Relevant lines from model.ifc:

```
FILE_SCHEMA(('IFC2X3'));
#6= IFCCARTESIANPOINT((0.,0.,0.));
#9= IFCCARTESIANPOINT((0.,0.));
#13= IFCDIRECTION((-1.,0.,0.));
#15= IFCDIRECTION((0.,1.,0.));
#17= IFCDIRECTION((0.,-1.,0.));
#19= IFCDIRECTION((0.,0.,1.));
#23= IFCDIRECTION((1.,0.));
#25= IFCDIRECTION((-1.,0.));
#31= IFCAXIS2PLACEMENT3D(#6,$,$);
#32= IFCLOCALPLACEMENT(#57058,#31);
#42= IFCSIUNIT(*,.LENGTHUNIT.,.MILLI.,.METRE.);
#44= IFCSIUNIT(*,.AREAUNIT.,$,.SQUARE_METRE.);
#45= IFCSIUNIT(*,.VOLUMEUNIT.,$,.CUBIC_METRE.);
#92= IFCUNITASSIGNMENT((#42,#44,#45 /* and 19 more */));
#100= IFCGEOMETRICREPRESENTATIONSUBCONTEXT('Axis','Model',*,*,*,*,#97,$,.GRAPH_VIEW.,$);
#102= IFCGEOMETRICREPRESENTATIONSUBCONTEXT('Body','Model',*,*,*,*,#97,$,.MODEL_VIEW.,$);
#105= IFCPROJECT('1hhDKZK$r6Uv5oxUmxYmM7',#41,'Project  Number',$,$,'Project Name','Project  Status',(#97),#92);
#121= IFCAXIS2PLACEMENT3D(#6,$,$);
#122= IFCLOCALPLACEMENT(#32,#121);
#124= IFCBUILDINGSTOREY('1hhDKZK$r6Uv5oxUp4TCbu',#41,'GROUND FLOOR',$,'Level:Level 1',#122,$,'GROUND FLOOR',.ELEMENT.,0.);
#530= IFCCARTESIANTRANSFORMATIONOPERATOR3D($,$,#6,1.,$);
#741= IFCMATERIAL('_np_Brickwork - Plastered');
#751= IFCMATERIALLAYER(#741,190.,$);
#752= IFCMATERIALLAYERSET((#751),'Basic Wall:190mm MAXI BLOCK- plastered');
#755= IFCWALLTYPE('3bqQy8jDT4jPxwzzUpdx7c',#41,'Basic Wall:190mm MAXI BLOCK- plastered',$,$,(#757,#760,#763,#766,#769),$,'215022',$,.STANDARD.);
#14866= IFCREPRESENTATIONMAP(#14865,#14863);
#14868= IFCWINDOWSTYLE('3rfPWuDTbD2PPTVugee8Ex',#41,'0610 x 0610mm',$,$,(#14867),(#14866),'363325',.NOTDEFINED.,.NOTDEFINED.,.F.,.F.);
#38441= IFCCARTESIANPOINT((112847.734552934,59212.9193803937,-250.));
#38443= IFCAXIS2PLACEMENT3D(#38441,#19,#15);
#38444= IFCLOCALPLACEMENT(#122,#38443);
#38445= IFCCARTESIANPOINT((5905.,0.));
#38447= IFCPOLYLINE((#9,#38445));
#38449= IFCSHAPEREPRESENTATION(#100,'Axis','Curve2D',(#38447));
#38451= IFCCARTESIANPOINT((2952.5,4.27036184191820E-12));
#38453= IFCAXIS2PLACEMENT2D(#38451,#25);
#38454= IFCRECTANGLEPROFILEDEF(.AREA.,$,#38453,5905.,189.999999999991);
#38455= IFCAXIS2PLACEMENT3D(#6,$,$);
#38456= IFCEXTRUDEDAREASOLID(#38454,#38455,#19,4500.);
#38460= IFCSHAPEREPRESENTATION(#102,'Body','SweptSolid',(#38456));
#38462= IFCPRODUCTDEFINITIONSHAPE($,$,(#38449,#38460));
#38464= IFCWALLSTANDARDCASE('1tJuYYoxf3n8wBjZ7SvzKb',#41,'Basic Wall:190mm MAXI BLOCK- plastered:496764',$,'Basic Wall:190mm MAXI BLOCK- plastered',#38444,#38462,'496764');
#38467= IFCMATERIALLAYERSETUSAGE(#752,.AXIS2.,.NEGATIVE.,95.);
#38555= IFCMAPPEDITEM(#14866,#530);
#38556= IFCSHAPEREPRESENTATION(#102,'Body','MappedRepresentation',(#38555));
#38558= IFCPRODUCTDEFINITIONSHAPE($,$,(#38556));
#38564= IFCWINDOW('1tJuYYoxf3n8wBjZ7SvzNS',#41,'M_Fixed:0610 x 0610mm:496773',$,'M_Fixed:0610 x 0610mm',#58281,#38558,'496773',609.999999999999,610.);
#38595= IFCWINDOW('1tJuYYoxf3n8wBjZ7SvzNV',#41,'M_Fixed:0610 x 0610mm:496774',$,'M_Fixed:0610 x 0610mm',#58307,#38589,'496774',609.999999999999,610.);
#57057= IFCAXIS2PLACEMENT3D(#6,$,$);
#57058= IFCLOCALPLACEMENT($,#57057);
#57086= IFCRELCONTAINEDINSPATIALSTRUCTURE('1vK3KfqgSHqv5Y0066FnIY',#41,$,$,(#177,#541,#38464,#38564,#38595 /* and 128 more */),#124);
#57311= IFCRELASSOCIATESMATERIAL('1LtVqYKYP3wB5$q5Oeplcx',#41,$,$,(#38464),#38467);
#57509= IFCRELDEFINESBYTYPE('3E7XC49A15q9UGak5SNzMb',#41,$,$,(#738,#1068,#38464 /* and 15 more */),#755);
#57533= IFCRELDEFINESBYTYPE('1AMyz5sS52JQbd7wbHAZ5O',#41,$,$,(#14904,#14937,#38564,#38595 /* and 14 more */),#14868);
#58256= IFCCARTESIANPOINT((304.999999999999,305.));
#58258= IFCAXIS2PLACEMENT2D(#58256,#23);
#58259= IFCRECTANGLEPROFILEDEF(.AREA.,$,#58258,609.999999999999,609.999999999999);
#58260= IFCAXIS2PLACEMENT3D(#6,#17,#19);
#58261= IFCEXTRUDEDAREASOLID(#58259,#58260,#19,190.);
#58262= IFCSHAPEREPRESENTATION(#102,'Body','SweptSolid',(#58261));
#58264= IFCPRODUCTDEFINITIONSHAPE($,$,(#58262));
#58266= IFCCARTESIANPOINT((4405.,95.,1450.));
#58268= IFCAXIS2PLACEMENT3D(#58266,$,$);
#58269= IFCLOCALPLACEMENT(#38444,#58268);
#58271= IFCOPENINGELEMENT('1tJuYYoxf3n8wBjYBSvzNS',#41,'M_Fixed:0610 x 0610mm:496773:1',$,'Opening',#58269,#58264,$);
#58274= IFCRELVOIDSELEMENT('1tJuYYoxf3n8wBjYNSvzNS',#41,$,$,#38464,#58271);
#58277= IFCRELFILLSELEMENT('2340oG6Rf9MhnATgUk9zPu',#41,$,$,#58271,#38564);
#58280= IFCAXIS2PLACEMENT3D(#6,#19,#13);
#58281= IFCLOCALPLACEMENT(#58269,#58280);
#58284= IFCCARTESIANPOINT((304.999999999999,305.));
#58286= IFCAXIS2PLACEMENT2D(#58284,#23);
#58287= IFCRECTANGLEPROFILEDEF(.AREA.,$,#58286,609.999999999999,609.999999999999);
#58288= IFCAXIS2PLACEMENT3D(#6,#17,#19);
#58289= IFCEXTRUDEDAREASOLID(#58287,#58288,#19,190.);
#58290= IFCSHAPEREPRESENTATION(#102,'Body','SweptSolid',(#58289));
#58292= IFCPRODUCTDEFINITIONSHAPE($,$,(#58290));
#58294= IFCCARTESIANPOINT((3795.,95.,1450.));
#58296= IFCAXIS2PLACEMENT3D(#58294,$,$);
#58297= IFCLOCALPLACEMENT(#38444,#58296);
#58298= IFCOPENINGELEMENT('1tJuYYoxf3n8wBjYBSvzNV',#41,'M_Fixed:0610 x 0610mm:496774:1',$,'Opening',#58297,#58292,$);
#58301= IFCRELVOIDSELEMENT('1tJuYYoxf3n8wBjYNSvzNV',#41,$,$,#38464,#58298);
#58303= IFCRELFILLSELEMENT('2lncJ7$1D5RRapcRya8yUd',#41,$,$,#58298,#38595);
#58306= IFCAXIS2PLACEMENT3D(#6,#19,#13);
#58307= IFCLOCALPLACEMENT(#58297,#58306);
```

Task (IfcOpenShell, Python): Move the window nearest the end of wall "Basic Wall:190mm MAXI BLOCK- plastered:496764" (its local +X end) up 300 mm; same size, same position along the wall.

```python
import numpy as np
import ifcopenshell
import ifcopenshell.api.geometry
import ifcopenshell.util.placement
import ifcopenshell.util.unit

model = ifcopenshell.open("model.ifc")
unit_scale = ifcopenshell.util.unit.calculate_unit_scale(model)

window = model.by_guid("1tJuYYoxf3n8wBjZ7SvzNS")
opening = window.FillsVoids[0].RelatingOpeningElement
dz = 300.0

shift = np.array([0.0, 0.0, dz])
# The window is placed relative to its opening, so it follows when the opening moves.
matrix = ifcopenshell.util.placement.get_local_placement(opening.ObjectPlacement)
matrix[:3, 3] += shift
ifcopenshell.api.geometry.edit_object_placement(
    model, product=opening, matrix=matrix, is_si=False, should_transform_children=True
)

print(f"moved by {dz * unit_scale:+.3f} m")

model.write("model_rev.ifc")
```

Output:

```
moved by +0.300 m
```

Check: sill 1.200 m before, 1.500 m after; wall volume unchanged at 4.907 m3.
